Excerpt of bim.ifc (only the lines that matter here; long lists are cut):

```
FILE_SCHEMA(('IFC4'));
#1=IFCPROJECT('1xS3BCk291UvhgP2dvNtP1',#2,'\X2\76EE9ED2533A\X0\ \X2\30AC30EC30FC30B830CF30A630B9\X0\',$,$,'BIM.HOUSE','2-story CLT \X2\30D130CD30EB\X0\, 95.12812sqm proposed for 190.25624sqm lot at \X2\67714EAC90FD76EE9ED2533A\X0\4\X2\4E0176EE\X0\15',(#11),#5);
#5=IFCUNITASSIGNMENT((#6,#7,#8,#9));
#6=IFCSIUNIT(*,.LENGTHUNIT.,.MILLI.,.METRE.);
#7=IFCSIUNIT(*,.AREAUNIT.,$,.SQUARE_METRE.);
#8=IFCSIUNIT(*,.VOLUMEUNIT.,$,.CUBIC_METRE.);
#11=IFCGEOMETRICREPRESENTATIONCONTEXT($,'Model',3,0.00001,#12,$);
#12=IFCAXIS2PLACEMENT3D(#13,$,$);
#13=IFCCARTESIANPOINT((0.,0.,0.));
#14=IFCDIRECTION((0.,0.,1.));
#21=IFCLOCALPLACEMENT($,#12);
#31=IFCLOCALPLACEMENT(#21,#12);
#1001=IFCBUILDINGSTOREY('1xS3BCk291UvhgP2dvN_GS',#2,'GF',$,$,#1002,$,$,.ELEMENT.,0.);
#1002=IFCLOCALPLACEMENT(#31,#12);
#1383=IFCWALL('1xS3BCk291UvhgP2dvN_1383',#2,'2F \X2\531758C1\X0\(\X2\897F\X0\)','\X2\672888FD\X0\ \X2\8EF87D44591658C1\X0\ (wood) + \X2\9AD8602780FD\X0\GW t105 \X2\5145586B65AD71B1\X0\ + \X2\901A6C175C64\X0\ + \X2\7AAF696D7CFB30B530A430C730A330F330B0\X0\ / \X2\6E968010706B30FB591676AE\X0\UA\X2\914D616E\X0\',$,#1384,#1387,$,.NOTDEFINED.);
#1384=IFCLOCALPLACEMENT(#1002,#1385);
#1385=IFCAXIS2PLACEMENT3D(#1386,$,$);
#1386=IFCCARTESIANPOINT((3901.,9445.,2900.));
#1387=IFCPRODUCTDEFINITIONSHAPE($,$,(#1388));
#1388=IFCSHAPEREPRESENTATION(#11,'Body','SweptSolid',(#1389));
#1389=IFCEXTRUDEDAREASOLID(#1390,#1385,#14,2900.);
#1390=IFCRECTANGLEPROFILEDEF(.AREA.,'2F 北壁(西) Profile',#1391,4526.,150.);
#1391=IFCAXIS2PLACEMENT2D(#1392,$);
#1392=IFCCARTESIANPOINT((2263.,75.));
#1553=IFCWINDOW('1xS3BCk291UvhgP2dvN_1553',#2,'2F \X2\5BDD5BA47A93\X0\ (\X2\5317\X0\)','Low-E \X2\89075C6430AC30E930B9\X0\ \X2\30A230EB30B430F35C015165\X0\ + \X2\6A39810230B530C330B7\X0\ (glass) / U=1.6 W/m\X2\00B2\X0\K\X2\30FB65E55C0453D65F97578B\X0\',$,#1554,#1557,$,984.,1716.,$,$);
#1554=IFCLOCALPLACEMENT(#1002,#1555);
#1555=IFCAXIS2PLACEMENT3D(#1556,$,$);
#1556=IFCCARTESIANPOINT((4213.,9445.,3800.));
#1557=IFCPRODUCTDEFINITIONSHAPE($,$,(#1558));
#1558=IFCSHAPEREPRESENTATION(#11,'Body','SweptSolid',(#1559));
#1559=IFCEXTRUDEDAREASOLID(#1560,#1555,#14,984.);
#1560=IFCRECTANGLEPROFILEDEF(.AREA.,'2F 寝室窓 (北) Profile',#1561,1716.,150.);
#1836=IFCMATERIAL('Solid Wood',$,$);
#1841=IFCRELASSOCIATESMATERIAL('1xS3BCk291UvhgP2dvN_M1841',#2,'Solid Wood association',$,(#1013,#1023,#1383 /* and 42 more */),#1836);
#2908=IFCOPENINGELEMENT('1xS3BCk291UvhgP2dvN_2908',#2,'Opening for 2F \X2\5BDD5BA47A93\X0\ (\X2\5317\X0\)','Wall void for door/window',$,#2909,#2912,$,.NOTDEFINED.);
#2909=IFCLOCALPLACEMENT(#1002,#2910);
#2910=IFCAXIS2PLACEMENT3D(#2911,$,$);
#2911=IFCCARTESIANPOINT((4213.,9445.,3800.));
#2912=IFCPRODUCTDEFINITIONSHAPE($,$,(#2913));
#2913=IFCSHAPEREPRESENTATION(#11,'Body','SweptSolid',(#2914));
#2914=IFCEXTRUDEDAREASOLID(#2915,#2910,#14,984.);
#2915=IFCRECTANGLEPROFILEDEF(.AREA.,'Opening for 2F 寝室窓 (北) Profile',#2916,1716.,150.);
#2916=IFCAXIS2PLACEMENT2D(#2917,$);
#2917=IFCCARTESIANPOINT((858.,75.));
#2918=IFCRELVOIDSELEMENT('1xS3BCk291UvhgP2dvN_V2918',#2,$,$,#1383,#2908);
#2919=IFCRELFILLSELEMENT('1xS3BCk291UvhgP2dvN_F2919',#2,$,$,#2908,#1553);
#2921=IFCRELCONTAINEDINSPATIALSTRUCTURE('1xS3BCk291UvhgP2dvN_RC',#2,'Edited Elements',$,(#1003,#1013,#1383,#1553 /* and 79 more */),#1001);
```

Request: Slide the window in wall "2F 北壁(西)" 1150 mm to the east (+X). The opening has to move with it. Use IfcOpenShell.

```python
import ifcopenshell
import ifcopenshell.api.geometry
import ifcopenshell.util.placement
import ifcopenshell.util.unit

model = ifcopenshell.open("bim.ifc")
unit_scale = ifcopenshell.util.unit.calculate_unit_scale(model)

window = model.by_guid("1xS3BCk291UvhgP2dvN_1553")
opening = window.FillsVoids[0].RelatingOpeningElement
wall = opening.VoidsElements[0].RelatingBuildingElement

wall_matrix = ifcopenshell.util.placement.get_local_placement(wall.ObjectPlacement)
shift = wall_matrix[:3, 0] * 1.15 / unit_scale
before = ifcopenshell.util.placement.get_local_placement(window.ObjectPlacement)[:3, 3].copy()

# The window is not placed relative to its opening, so move both.
for product in (opening, window):
    matrix = ifcopenshell.util.placement.get_local_placement(product.ObjectPlacement)
    matrix[:3, 3] += shift
    ifcopenshell.api.geometry.edit_object_placement(model, product=product, matrix=matrix, is_si=False)

after = ifcopenshell.util.placement.get_local_placement(window.ObjectPlacement)[:3, 3]
print("window moved by", (after - before).round(3) + 0.0)

model.write("bim_edited.ifc")
```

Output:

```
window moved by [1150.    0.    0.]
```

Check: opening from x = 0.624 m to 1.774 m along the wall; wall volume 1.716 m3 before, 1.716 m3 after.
